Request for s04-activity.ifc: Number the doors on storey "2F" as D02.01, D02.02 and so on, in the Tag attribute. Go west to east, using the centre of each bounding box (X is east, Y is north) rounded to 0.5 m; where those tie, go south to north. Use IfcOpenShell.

First a look at what the model holds.

```python
import ifcopenshell
import ifcopenshell.util.element
import ifcopenshell.util.placement

model = ifcopenshell.open("s04-activity.ifc")
print(model.schema)
storey = next(s for s in model.by_type("IfcBuildingStorey") if s.Name == "2F")
doors = [e for e in ifcopenshell.util.element.get_decomposition(storey) if e.is_a("IfcDoor")]
for e in sorted(doors, key=lambda e: e.id()):
    origin = ifcopenshell.util.placement.get_local_placement(e.ObjectPlacement)[:3, 3]
    print(e.id(), e.Tag, e.Name, origin.round(2) + 0.0, sep=" | ")
```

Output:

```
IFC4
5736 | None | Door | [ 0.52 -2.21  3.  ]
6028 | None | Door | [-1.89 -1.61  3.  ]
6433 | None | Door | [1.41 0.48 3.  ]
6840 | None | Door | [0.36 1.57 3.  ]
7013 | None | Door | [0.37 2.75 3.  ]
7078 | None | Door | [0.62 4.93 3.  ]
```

```python
import ifcopenshell
import ifcopenshell.geom
import ifcopenshell.util.element
import ifcopenshell.util.shape

model = ifcopenshell.open("s04-activity.ifc")
settings = ifcopenshell.geom.settings()
settings.set("use-world-coords", True)


def centre(element):
    shape = ifcopenshell.geom.create_shape(settings, element)
    return ifcopenshell.util.shape.get_bbox_centroid(shape.geometry)


storey = next(s for s in model.by_type("IfcBuildingStorey") if s.Name == "2F")
doors = [e for e in ifcopenshell.util.element.get_decomposition(storey) if e.is_a("IfcDoor")]

# Insertion points can sit at a corner or the storey origin, so sort by the geometry (in metres).
centres = {e: centre(e) for e in doors}
doors.sort(key=lambda e: (round(centres[e][0] / 0.5), centres[e][1]))

for i, e in enumerate(doors, start=1):
    number = f"D02.{i:02d}"
    e.Tag = number
    print(e.id(), number)

model.write("s04-activity-out.ifc")
```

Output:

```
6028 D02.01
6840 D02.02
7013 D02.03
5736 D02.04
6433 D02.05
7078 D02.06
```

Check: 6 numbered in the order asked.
